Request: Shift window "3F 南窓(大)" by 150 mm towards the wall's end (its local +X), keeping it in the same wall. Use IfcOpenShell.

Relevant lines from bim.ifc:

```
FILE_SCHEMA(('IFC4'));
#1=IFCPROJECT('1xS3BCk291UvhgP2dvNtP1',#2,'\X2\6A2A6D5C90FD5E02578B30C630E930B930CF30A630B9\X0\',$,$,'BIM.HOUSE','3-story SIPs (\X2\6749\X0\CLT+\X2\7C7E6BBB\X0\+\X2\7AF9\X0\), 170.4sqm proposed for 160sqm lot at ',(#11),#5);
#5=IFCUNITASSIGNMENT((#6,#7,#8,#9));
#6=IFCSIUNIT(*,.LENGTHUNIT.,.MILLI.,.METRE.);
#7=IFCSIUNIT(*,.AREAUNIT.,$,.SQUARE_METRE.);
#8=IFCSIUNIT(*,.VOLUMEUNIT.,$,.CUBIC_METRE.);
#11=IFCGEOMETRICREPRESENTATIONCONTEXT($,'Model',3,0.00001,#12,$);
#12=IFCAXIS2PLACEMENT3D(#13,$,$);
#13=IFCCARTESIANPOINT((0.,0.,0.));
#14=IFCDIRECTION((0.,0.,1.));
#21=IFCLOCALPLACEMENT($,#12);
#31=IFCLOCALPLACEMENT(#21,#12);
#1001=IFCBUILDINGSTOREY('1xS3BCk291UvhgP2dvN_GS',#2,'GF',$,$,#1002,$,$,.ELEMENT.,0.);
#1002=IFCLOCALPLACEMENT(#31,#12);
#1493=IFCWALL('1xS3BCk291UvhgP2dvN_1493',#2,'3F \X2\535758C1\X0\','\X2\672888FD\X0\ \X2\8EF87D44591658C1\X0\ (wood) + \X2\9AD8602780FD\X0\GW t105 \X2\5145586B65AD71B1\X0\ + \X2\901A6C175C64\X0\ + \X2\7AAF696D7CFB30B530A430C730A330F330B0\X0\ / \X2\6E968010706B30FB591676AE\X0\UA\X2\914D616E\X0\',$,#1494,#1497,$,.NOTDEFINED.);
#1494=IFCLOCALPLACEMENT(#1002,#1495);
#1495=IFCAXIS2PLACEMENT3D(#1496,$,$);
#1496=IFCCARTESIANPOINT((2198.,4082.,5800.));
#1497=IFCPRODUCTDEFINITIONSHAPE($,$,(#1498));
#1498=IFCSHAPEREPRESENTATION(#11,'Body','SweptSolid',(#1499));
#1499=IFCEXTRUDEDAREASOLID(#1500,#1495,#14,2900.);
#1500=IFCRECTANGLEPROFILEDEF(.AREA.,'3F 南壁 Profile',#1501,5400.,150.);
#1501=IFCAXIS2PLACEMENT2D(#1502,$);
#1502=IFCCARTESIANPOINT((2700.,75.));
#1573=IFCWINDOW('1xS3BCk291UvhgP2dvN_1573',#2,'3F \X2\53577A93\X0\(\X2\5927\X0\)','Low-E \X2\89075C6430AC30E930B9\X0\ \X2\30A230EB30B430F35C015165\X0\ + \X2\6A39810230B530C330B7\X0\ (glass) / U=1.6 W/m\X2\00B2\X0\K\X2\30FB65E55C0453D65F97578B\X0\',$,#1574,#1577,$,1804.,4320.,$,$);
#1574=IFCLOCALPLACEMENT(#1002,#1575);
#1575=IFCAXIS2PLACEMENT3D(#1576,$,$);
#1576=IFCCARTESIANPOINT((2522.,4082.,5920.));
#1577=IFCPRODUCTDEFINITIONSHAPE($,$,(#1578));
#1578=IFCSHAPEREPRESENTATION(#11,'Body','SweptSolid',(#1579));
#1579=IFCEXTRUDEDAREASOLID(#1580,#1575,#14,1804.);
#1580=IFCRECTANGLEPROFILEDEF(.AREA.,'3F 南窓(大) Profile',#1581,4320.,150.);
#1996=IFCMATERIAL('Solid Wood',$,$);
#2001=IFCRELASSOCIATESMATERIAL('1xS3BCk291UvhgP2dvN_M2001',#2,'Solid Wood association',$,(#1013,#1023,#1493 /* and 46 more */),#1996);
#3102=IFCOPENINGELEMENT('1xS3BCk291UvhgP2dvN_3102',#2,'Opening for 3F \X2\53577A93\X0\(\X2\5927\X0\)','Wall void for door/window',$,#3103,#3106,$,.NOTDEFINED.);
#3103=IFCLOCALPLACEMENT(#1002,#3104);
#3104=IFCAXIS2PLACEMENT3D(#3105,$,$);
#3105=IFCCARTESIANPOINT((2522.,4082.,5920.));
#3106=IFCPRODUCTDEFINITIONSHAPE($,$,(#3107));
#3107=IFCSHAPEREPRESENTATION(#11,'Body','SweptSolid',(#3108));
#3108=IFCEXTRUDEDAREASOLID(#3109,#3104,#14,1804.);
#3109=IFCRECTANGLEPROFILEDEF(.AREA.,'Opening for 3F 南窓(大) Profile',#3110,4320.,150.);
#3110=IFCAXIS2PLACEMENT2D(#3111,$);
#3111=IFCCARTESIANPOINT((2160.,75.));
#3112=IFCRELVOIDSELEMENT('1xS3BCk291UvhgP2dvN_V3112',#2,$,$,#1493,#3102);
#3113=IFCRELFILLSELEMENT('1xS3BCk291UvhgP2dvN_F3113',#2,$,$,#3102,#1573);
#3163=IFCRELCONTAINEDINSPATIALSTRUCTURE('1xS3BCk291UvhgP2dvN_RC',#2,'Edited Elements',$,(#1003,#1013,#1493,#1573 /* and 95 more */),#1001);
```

```python
import ifcopenshell
import ifcopenshell.api.geometry
import ifcopenshell.util.placement

model = ifcopenshell.open("bim.ifc")

window = model.by_guid("1xS3BCk291UvhgP2dvN_1573")
opening = window.FillsVoids[0].RelatingOpeningElement
wall = opening.VoidsElements[0].RelatingBuildingElement

wall_matrix = ifcopenshell.util.placement.get_local_placement(wall.ObjectPlacement)
shift = wall_matrix[:3, 0] * 150.0
before = ifcopenshell.util.placement.get_local_placement(window.ObjectPlacement)[:3, 3].copy()

# The window is not placed relative to its opening, so move both.
for product in (opening, window):
    matrix = ifcopenshell.util.placement.get_local_placement(product.ObjectPlacement)
    matrix[:3, 3] += shift
    ifcopenshell.api.geometry.edit_object_placement(model, product=product, matrix=matrix, is_si=False)

after = ifcopenshell.util.placement.get_local_placement(window.ObjectPlacement)[:3, 3]
print("window moved by", (after - before).round(3) + 0.0)

model.write("bim_rev.ifc")
```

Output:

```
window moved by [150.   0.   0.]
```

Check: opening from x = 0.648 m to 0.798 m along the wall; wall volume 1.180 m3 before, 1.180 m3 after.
